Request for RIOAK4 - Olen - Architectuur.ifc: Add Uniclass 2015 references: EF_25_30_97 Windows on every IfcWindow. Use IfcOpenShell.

First a look at what the model holds.

```python
import ifcopenshell

model = ifcopenshell.open("RIOAK4 - Olen - Architectuur.ifc")
print(model.schema)
print("classifications:", [c.Name for c in model.by_type("IfcClassification")])
for ifc_class in ("IfcDoor", "IfcRoof", "IfcStair", "IfcWall", "IfcWindow"):
    print(ifc_class, len(model.by_type(ifc_class)))
```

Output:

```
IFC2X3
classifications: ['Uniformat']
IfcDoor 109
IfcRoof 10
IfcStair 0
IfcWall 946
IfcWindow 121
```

```python
import ifcopenshell
import ifcopenshell.api.classification

model = ifcopenshell.open("RIOAK4 - Olen - Architectuur.ifc")

# IFC2X3 requires Source and Edition and has no link from the project to the system.
system = model.create_entity("IfcClassification", Source="NBS", Edition="2015", Name="Uniclass 2015")

codes = {
    "IfcWindow": ("EF_25_30_97", "Windows"),
}
for ifc_class, (code, name) in codes.items():
    products = model.by_type(ifc_class)
    ifcopenshell.api.classification.add_reference(
        model, products=products, classification=system, identification=code, name=name
    )
    print(code, len(products))

model.write("RIOAK4 - Olen - Architectuur_edited.ifc")
```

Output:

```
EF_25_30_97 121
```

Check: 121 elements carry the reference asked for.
